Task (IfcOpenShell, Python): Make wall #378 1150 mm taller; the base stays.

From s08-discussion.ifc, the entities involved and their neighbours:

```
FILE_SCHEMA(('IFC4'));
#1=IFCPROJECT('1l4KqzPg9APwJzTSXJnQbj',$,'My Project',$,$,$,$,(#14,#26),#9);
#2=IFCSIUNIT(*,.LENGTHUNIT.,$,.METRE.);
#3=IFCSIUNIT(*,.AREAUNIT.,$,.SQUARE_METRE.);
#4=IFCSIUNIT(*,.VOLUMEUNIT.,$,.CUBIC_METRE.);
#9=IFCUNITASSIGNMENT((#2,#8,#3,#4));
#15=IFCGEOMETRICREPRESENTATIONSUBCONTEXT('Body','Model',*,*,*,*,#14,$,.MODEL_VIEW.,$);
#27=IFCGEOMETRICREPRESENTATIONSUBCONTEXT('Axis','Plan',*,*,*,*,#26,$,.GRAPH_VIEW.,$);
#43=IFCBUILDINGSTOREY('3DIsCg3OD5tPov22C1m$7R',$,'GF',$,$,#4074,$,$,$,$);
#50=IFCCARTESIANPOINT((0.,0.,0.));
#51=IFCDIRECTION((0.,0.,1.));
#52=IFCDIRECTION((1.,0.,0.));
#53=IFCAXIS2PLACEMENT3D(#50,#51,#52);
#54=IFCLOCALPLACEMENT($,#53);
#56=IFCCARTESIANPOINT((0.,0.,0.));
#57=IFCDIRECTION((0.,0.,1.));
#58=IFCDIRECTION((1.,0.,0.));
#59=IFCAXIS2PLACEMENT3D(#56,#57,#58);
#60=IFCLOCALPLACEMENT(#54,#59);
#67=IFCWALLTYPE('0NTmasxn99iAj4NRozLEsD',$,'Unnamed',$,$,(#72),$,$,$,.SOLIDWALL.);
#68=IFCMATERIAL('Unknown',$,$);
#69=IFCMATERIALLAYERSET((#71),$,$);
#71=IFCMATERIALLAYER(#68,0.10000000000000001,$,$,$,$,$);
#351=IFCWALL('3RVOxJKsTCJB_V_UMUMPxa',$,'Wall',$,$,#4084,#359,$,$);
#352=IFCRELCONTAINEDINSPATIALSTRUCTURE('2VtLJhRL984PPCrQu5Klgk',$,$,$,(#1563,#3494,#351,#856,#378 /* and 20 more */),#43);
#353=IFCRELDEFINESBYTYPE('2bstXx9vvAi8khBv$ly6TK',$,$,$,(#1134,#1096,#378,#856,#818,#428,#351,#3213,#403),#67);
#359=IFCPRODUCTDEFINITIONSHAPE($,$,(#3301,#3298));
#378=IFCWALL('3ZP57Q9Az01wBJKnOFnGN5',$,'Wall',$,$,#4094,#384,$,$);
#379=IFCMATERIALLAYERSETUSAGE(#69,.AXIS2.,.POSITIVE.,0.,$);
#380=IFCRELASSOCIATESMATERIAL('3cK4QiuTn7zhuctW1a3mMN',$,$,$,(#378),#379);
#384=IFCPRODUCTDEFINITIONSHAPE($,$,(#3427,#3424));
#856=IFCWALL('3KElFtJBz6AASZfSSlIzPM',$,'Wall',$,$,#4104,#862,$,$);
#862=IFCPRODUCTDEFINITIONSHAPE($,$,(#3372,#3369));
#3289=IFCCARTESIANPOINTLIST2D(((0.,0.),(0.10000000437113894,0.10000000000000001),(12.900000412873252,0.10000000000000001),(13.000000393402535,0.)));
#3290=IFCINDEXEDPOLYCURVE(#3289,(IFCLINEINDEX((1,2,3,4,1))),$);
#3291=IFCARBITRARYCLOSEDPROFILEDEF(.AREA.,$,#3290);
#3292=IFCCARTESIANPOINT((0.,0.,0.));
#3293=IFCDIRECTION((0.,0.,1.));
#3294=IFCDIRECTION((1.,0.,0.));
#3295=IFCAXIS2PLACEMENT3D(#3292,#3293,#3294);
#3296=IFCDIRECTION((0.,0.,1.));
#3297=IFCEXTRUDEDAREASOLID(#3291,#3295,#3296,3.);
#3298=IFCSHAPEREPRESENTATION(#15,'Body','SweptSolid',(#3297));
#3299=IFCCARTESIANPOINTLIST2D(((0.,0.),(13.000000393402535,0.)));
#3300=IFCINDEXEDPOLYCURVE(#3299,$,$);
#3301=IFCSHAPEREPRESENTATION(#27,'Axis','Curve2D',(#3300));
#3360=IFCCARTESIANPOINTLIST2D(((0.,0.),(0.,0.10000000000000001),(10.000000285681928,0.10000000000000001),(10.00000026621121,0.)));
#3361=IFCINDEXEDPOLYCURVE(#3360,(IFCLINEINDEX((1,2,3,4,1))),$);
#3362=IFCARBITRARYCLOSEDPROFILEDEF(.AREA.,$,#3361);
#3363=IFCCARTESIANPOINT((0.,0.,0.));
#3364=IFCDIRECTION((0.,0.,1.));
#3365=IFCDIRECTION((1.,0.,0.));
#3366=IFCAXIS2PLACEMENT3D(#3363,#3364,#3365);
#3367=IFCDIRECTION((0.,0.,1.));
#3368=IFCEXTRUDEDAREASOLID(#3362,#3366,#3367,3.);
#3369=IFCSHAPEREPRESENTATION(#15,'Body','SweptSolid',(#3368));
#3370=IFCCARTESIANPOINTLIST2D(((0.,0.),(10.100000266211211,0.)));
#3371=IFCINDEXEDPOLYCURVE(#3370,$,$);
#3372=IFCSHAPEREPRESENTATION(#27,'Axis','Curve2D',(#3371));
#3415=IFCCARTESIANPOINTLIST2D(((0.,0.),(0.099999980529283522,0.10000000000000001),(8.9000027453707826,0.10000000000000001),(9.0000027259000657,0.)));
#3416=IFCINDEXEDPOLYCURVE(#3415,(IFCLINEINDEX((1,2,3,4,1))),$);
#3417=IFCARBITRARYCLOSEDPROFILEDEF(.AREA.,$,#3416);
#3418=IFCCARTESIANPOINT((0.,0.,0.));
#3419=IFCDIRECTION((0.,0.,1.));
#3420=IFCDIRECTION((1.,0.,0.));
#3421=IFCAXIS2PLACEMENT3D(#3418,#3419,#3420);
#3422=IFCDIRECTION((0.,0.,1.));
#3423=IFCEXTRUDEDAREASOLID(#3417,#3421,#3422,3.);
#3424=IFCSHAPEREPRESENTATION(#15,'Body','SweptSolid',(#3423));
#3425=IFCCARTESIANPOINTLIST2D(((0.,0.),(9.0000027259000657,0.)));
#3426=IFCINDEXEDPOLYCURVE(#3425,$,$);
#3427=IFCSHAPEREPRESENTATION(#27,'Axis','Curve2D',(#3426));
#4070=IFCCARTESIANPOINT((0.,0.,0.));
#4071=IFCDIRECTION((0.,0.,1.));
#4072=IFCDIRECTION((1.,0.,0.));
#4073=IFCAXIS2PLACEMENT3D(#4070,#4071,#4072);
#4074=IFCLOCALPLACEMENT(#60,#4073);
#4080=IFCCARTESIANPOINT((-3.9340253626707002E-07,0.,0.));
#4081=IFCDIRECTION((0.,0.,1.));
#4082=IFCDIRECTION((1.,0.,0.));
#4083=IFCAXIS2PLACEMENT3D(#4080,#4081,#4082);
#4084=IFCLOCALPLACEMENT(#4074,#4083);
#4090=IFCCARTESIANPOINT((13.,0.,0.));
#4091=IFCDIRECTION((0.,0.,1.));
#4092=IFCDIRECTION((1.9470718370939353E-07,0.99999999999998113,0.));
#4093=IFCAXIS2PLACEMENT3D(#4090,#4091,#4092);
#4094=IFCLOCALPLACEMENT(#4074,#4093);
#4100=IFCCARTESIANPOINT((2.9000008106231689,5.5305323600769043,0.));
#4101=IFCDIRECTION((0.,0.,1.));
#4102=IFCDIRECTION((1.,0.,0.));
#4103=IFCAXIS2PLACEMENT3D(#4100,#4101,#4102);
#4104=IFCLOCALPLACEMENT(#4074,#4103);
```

```python
import ifcopenshell
import ifcopenshell.geom
import ifcopenshell.util.representation
import ifcopenshell.util.shape

model = ifcopenshell.open("s08-discussion.ifc")
settings = ifcopenshell.geom.settings()


def volume(element):
    """Net volume in cubic metres, openings subtracted."""
    shape = ifcopenshell.geom.create_shape(settings, element)
    return ifcopenshell.util.shape.get_volume(shape.geometry)


wall = model.by_id(378)
before = volume(wall)

body = ifcopenshell.util.representation.get_representation(wall, "Model", "Body")
solid = body.Items[0]
old_height = solid.Depth
solid.Depth += 1.15
after = volume(wall)

print(f"height {old_height:g} -> {solid.Depth:g}, volume {before:.3f} -> {after:.3f} m3")

model.write("s08-discussion_updated.ifc")
```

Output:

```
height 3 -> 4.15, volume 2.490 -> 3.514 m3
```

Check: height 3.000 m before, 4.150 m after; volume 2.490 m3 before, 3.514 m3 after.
